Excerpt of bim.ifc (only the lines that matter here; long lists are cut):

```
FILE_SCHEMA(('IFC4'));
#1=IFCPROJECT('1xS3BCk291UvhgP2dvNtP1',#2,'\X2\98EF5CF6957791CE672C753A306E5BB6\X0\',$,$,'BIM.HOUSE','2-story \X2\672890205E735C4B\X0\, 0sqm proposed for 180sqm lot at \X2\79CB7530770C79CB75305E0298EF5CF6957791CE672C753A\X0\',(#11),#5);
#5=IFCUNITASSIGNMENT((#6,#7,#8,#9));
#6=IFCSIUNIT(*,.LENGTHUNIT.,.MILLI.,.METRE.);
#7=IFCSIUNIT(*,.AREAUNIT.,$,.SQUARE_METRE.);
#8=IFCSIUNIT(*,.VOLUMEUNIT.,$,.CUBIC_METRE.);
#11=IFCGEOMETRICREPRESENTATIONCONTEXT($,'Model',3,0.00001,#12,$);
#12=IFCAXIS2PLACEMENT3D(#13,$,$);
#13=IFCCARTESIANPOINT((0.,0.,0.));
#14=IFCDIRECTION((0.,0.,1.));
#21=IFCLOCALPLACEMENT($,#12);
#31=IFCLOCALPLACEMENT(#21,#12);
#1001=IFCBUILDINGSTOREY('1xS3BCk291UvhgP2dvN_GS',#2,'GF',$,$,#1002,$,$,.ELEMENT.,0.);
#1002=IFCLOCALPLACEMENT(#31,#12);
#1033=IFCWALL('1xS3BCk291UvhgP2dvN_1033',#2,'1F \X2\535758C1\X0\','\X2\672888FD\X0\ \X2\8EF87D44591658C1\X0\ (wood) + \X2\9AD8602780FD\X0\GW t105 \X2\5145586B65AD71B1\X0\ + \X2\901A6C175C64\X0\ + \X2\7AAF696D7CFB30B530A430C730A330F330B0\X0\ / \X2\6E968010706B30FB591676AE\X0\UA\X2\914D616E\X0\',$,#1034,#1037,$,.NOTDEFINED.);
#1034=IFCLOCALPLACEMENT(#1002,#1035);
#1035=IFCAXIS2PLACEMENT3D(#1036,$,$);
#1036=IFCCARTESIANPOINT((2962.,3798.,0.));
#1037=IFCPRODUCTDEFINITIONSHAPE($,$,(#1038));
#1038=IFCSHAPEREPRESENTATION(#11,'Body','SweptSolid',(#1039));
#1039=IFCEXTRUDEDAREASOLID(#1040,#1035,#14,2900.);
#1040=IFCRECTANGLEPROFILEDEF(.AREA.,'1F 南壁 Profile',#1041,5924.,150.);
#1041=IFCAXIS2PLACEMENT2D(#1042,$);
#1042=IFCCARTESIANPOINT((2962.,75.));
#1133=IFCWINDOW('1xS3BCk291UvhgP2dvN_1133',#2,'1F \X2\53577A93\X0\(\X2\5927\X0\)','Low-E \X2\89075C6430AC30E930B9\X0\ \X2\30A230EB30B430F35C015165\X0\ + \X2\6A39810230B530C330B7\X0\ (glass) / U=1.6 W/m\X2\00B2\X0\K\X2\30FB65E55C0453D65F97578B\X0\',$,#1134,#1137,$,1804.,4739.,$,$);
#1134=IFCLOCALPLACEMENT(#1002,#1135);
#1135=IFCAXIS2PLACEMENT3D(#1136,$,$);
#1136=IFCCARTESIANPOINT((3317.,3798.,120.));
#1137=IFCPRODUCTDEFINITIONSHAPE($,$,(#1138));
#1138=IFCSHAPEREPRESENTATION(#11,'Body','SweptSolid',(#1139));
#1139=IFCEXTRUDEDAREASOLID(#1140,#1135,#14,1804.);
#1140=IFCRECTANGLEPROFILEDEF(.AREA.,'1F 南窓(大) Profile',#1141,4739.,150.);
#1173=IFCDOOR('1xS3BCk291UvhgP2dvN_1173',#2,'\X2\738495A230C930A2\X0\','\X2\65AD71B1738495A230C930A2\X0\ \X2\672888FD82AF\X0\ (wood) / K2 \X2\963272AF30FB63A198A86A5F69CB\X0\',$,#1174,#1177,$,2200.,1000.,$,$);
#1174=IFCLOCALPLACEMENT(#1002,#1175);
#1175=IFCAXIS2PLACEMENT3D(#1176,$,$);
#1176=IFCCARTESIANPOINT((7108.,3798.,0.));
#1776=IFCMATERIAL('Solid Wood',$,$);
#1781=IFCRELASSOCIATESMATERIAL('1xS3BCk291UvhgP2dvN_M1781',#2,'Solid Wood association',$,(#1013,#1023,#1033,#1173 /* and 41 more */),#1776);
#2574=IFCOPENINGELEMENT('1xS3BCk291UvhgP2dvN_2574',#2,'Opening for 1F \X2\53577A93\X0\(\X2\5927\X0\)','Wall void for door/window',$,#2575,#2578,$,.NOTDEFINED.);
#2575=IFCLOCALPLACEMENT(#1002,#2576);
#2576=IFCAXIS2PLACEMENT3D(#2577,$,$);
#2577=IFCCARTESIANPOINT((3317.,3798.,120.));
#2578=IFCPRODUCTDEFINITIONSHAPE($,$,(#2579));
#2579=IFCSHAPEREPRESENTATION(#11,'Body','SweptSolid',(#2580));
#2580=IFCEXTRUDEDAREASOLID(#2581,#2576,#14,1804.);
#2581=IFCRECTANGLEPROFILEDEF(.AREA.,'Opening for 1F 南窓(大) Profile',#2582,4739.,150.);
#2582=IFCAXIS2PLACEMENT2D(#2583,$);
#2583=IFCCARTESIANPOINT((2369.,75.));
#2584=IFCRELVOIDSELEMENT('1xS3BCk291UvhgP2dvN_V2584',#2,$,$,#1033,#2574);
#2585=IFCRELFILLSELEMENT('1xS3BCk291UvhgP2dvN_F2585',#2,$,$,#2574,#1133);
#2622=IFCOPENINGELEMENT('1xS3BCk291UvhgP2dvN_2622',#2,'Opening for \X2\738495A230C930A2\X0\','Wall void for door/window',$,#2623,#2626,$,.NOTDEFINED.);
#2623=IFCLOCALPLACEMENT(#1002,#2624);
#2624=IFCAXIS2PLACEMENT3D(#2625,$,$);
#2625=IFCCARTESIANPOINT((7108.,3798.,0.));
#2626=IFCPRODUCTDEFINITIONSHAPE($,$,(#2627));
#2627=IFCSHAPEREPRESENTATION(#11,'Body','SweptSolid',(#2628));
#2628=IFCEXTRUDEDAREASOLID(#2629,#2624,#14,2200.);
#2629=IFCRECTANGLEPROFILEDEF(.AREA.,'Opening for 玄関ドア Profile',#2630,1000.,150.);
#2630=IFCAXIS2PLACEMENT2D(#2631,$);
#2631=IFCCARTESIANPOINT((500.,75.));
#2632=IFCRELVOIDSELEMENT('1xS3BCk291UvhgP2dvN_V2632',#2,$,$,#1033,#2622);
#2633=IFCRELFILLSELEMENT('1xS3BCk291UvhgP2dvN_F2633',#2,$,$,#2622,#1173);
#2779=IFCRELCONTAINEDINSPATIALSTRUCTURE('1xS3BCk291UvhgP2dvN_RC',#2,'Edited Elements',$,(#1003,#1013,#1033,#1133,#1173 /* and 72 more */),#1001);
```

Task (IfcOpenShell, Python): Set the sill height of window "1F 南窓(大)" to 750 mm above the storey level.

```python
import numpy as np
import ifcopenshell
import ifcopenshell.api.geometry
import ifcopenshell.geom
import ifcopenshell.util.element
import ifcopenshell.util.placement
import ifcopenshell.util.shape
import ifcopenshell.util.unit

model = ifcopenshell.open("bim.ifc")
unit_scale = ifcopenshell.util.unit.calculate_unit_scale(model)

window = model.by_id(1133)
opening = window.FillsVoids[0].RelatingOpeningElement
storey = ifcopenshell.util.element.get_container(window, ifc_class="IfcBuildingStorey")
level = ifcopenshell.util.placement.get_local_placement(storey.ObjectPlacement)[2, 3]

# The opening's origin need not be at the sill, so measure its lowest point.
shape = ifcopenshell.geom.create_shape(ifcopenshell.geom.settings(), opening)
bottom = ifcopenshell.util.shape.get_shape_bottom_elevation(shape, shape.geometry) / unit_scale
dz = level + 0.75 / unit_scale - bottom

shift = np.array([0.0, 0.0, dz])
# The window is not placed relative to its opening, so move both.
for product in (opening, window):
    matrix = ifcopenshell.util.placement.get_local_placement(product.ObjectPlacement)
    matrix[:3, 3] += shift
    ifcopenshell.api.geometry.edit_object_placement(model, product=product, matrix=matrix, is_si=False)

print(f"moved by {dz * unit_scale:+.3f} m")

model.write("bim_rev.ifc")
```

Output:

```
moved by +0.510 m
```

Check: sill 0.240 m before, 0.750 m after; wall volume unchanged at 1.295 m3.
